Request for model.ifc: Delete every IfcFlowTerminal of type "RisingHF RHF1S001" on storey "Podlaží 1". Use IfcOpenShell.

First a look at what the model holds.

```python
import ifcopenshell
import ifcopenshell.util.element

model = ifcopenshell.open("model.ifc")
print(model.schema)
storey = next(s for s in model.by_type("IfcBuildingStorey") if s.Name == "Podlaží 1")
terminals = [e for e in ifcopenshell.util.element.get_decomposition(storey) if e.is_a("IfcFlowTerminal")]
seen = {}
for e in terminals:
    element_type = ifcopenshell.util.element.get_type(e)
    name = element_type.Name if element_type not in (None, e) else None
    seen[name] = seen.get(name, 0) + 1
for name, count in sorted(seen.items(), key=str):
    print(count, "x", name)
```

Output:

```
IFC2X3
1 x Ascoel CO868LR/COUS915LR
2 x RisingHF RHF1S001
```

```python
import ifcopenshell
import ifcopenshell.api.root
import ifcopenshell.util.element

model = ifcopenshell.open("model.ifc")

storey = next(s for s in model.by_type("IfcBuildingStorey") if s.Name == "Podlaží 1")
terminals = [e for e in ifcopenshell.util.element.get_decomposition(storey) if e.is_a("IfcFlowTerminal")]
targets = [e for e in terminals if (t := ifcopenshell.util.element.get_type(e)) not in (None, e) and t.Name == "RisingHF RHF1S001"]

for e in targets:
    ifcopenshell.api.root.remove_product(model, product=e)
print(len(targets), "removed")

model.write("model_v2.ifc")
```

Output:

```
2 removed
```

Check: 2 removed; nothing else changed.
